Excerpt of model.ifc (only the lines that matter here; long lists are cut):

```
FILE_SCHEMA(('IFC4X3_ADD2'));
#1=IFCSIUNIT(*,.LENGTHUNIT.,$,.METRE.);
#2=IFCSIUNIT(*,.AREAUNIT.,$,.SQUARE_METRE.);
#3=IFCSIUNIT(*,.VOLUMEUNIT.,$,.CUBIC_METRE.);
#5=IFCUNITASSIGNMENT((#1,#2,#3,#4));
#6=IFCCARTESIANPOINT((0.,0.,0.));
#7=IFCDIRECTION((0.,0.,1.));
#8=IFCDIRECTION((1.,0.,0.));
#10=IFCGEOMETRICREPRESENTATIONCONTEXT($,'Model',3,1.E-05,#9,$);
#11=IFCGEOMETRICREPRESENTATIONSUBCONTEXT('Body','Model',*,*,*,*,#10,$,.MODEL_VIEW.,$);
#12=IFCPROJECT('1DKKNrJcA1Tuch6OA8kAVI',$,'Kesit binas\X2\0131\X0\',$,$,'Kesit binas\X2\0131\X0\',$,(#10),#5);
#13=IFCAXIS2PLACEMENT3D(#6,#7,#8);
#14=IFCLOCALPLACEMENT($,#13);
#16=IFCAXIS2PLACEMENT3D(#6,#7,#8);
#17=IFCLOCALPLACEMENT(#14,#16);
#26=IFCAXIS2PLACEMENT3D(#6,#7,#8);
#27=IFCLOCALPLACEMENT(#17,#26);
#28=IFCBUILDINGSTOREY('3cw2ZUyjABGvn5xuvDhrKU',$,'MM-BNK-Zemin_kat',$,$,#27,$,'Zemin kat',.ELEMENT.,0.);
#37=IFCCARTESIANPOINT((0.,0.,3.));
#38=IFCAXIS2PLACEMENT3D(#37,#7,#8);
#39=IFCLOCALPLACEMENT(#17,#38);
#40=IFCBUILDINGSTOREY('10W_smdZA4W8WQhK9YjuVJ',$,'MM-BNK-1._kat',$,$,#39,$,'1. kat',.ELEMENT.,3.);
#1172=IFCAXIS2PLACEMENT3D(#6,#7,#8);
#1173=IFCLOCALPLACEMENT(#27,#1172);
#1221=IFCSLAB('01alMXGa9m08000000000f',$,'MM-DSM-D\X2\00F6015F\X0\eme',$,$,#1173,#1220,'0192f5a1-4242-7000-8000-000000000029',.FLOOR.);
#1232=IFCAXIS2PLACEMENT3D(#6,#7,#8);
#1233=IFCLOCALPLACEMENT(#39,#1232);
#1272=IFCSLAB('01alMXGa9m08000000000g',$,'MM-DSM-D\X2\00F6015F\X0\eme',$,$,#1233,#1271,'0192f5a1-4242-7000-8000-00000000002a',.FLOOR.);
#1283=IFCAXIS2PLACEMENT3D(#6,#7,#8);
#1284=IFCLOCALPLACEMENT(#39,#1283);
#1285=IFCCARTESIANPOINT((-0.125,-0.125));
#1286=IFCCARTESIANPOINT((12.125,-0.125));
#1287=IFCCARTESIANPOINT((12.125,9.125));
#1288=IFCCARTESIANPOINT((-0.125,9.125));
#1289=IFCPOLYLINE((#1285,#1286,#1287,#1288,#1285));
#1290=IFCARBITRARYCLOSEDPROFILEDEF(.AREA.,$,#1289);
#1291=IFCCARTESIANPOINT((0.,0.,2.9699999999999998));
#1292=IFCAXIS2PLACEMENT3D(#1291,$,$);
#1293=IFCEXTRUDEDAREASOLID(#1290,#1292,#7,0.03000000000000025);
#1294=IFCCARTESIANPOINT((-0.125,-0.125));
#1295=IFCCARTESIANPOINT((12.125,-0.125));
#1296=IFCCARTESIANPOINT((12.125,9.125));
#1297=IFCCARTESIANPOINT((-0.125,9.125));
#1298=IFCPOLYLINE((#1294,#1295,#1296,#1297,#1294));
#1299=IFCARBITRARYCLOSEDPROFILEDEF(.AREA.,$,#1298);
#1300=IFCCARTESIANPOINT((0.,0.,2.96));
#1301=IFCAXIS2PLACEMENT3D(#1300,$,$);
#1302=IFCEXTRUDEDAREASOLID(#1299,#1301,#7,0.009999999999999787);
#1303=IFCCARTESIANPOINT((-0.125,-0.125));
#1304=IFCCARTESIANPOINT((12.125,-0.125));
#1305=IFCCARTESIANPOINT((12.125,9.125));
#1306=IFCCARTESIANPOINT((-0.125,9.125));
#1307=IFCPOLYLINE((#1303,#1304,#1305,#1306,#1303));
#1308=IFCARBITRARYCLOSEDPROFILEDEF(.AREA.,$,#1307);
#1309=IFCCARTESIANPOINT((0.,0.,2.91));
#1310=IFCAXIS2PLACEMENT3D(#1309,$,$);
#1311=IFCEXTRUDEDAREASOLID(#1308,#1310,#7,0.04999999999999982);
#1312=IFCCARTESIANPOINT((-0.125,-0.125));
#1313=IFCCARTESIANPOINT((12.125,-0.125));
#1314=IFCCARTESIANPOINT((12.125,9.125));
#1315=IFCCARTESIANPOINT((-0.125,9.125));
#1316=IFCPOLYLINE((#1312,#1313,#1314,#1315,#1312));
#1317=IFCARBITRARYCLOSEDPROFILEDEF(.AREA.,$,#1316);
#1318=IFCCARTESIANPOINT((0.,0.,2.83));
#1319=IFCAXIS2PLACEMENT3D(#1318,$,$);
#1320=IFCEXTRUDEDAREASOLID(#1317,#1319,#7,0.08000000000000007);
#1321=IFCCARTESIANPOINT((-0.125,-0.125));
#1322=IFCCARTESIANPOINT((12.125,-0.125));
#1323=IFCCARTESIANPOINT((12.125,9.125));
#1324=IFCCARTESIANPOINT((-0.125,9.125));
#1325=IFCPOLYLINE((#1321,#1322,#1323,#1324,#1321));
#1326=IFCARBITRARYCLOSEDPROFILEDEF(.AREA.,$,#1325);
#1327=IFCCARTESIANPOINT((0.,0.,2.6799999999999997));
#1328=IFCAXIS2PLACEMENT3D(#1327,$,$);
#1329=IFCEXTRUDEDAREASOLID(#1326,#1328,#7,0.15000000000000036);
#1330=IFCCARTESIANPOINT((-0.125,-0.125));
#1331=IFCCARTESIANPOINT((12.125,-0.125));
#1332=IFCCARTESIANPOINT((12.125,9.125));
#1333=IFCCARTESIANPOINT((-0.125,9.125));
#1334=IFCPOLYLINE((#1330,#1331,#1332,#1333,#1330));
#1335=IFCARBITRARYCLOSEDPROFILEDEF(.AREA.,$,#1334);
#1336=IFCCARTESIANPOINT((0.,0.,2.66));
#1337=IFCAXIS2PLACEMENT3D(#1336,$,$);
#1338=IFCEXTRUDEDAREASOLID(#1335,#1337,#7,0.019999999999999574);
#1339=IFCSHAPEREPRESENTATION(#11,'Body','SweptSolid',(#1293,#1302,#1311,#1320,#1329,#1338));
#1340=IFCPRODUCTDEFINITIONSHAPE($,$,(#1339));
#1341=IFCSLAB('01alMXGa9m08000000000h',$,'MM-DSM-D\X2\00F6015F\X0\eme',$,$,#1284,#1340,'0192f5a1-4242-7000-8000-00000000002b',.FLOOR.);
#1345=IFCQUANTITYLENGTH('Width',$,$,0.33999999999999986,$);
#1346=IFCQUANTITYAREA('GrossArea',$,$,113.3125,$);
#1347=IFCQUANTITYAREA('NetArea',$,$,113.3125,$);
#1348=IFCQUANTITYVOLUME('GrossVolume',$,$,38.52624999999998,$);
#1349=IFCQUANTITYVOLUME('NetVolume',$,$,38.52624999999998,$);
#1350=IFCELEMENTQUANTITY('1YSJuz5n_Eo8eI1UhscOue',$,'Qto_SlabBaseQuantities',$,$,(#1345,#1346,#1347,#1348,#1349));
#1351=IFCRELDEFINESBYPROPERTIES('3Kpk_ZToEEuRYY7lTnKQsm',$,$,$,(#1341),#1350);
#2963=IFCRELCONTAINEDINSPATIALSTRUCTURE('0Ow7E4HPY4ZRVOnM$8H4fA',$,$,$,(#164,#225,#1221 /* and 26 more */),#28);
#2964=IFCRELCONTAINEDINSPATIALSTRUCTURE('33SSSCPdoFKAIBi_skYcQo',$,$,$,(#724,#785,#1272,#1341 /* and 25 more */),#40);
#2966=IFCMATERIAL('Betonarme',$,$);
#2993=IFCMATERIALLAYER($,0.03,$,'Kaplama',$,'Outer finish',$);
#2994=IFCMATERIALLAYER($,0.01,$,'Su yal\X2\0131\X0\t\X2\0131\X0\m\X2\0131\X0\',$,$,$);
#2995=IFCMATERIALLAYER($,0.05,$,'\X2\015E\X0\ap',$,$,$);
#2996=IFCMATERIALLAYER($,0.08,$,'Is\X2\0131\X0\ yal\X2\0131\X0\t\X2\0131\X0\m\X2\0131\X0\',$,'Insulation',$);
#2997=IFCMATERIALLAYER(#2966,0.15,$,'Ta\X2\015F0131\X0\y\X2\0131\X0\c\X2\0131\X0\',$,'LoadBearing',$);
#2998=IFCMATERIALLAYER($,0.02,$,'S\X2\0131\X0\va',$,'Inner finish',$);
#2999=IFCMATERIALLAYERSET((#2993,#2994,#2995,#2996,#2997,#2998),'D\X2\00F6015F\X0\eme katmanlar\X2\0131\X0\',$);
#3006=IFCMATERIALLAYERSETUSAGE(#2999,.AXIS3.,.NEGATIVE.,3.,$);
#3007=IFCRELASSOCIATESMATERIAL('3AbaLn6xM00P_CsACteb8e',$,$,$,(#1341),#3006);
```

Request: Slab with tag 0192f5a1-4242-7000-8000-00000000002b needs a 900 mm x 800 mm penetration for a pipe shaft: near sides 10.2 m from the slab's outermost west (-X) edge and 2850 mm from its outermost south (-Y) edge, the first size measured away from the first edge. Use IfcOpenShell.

```python
import numpy as np
import ifcopenshell
import ifcopenshell.api.feature
import ifcopenshell.api.geometry
import ifcopenshell.api.pset
import ifcopenshell.api.root
import ifcopenshell.geom
import ifcopenshell.util.element
import ifcopenshell.util.placement
import ifcopenshell.util.representation
import ifcopenshell.util.shape
import ifcopenshell.util.unit

model = ifcopenshell.open("model.ifc")
unit_scale = ifcopenshell.util.unit.calculate_unit_scale(model)
area_scale = ifcopenshell.util.unit.calculate_unit_scale(model, "AREAUNIT")
volume_scale = ifcopenshell.util.unit.calculate_unit_scale(model, "VOLUMEUNIT")
settings = ifcopenshell.geom.settings()


def volume(element):
    """Net volume in cubic metres, openings subtracted."""
    shape = ifcopenshell.geom.create_shape(settings, element)
    return ifcopenshell.util.shape.get_volume(shape.geometry)


slab = model.by_guid("01alMXGa9m08000000000h")
before = volume(slab)

# Extent in the slab's own axes, in metres. The edges named are its -X and -Y sides.
slab_shape = ifcopenshell.geom.create_shape(settings, slab)
vertices = ifcopenshell.util.shape.get_vertices(slab_shape.geometry)
x_min, y_min, bottom = vertices.min(axis=0)
top = vertices[:, 2].max()

opening = ifcopenshell.api.root.create_entity(model, ifc_class="IfcOpeningElement", name="Pipe shaft opening", predefined_type="OPENING")
context = ifcopenshell.util.representation.get_context(model, "Model", "Body", "MODEL_VIEW")
width, depth = 0.9, 0.8
outline = [(0.0, 0.0), (width, 0.0), (width, depth), (0.0, depth), (0.0, 0.0)]
# Overshoot both faces by 50 mm so the cut is clean.
shape = ifcopenshell.api.geometry.add_slab_representation(
    model, context=context, depth=top - bottom + 0.1, polyline=outline
)
ifcopenshell.api.geometry.assign_representation(model, product=opening, representation=shape)

matrix = ifcopenshell.util.placement.get_local_placement(slab.ObjectPlacement)
matrix[:, 3] = matrix @ np.append(np.array([x_min + 10.2, y_min + 2.85, bottom - 0.05]) / unit_scale, 1.0)
ifcopenshell.api.geometry.edit_object_placement(model, product=opening, matrix=matrix, is_si=False)
ifcopenshell.api.feature.add_feature(model, feature=opening, element=slab)

after = volume(slab)

# Update the slab's stored quantities.
qto = model.by_id(ifcopenshell.util.element.get_pset(slab, "Qto_SlabBaseQuantities", should_inherit=False)["id"])
ifcopenshell.api.pset.edit_qto(model, qto=qto, properties={
    "NetArea": after / (top - bottom) / area_scale,
    "NetVolume": after / volume_scale,
})

print(f"slab volume {before:.3f} -> {after:.3f} m3")

model.write("model_rev.ifc")
```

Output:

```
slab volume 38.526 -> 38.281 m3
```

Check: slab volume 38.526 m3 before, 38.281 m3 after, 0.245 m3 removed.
